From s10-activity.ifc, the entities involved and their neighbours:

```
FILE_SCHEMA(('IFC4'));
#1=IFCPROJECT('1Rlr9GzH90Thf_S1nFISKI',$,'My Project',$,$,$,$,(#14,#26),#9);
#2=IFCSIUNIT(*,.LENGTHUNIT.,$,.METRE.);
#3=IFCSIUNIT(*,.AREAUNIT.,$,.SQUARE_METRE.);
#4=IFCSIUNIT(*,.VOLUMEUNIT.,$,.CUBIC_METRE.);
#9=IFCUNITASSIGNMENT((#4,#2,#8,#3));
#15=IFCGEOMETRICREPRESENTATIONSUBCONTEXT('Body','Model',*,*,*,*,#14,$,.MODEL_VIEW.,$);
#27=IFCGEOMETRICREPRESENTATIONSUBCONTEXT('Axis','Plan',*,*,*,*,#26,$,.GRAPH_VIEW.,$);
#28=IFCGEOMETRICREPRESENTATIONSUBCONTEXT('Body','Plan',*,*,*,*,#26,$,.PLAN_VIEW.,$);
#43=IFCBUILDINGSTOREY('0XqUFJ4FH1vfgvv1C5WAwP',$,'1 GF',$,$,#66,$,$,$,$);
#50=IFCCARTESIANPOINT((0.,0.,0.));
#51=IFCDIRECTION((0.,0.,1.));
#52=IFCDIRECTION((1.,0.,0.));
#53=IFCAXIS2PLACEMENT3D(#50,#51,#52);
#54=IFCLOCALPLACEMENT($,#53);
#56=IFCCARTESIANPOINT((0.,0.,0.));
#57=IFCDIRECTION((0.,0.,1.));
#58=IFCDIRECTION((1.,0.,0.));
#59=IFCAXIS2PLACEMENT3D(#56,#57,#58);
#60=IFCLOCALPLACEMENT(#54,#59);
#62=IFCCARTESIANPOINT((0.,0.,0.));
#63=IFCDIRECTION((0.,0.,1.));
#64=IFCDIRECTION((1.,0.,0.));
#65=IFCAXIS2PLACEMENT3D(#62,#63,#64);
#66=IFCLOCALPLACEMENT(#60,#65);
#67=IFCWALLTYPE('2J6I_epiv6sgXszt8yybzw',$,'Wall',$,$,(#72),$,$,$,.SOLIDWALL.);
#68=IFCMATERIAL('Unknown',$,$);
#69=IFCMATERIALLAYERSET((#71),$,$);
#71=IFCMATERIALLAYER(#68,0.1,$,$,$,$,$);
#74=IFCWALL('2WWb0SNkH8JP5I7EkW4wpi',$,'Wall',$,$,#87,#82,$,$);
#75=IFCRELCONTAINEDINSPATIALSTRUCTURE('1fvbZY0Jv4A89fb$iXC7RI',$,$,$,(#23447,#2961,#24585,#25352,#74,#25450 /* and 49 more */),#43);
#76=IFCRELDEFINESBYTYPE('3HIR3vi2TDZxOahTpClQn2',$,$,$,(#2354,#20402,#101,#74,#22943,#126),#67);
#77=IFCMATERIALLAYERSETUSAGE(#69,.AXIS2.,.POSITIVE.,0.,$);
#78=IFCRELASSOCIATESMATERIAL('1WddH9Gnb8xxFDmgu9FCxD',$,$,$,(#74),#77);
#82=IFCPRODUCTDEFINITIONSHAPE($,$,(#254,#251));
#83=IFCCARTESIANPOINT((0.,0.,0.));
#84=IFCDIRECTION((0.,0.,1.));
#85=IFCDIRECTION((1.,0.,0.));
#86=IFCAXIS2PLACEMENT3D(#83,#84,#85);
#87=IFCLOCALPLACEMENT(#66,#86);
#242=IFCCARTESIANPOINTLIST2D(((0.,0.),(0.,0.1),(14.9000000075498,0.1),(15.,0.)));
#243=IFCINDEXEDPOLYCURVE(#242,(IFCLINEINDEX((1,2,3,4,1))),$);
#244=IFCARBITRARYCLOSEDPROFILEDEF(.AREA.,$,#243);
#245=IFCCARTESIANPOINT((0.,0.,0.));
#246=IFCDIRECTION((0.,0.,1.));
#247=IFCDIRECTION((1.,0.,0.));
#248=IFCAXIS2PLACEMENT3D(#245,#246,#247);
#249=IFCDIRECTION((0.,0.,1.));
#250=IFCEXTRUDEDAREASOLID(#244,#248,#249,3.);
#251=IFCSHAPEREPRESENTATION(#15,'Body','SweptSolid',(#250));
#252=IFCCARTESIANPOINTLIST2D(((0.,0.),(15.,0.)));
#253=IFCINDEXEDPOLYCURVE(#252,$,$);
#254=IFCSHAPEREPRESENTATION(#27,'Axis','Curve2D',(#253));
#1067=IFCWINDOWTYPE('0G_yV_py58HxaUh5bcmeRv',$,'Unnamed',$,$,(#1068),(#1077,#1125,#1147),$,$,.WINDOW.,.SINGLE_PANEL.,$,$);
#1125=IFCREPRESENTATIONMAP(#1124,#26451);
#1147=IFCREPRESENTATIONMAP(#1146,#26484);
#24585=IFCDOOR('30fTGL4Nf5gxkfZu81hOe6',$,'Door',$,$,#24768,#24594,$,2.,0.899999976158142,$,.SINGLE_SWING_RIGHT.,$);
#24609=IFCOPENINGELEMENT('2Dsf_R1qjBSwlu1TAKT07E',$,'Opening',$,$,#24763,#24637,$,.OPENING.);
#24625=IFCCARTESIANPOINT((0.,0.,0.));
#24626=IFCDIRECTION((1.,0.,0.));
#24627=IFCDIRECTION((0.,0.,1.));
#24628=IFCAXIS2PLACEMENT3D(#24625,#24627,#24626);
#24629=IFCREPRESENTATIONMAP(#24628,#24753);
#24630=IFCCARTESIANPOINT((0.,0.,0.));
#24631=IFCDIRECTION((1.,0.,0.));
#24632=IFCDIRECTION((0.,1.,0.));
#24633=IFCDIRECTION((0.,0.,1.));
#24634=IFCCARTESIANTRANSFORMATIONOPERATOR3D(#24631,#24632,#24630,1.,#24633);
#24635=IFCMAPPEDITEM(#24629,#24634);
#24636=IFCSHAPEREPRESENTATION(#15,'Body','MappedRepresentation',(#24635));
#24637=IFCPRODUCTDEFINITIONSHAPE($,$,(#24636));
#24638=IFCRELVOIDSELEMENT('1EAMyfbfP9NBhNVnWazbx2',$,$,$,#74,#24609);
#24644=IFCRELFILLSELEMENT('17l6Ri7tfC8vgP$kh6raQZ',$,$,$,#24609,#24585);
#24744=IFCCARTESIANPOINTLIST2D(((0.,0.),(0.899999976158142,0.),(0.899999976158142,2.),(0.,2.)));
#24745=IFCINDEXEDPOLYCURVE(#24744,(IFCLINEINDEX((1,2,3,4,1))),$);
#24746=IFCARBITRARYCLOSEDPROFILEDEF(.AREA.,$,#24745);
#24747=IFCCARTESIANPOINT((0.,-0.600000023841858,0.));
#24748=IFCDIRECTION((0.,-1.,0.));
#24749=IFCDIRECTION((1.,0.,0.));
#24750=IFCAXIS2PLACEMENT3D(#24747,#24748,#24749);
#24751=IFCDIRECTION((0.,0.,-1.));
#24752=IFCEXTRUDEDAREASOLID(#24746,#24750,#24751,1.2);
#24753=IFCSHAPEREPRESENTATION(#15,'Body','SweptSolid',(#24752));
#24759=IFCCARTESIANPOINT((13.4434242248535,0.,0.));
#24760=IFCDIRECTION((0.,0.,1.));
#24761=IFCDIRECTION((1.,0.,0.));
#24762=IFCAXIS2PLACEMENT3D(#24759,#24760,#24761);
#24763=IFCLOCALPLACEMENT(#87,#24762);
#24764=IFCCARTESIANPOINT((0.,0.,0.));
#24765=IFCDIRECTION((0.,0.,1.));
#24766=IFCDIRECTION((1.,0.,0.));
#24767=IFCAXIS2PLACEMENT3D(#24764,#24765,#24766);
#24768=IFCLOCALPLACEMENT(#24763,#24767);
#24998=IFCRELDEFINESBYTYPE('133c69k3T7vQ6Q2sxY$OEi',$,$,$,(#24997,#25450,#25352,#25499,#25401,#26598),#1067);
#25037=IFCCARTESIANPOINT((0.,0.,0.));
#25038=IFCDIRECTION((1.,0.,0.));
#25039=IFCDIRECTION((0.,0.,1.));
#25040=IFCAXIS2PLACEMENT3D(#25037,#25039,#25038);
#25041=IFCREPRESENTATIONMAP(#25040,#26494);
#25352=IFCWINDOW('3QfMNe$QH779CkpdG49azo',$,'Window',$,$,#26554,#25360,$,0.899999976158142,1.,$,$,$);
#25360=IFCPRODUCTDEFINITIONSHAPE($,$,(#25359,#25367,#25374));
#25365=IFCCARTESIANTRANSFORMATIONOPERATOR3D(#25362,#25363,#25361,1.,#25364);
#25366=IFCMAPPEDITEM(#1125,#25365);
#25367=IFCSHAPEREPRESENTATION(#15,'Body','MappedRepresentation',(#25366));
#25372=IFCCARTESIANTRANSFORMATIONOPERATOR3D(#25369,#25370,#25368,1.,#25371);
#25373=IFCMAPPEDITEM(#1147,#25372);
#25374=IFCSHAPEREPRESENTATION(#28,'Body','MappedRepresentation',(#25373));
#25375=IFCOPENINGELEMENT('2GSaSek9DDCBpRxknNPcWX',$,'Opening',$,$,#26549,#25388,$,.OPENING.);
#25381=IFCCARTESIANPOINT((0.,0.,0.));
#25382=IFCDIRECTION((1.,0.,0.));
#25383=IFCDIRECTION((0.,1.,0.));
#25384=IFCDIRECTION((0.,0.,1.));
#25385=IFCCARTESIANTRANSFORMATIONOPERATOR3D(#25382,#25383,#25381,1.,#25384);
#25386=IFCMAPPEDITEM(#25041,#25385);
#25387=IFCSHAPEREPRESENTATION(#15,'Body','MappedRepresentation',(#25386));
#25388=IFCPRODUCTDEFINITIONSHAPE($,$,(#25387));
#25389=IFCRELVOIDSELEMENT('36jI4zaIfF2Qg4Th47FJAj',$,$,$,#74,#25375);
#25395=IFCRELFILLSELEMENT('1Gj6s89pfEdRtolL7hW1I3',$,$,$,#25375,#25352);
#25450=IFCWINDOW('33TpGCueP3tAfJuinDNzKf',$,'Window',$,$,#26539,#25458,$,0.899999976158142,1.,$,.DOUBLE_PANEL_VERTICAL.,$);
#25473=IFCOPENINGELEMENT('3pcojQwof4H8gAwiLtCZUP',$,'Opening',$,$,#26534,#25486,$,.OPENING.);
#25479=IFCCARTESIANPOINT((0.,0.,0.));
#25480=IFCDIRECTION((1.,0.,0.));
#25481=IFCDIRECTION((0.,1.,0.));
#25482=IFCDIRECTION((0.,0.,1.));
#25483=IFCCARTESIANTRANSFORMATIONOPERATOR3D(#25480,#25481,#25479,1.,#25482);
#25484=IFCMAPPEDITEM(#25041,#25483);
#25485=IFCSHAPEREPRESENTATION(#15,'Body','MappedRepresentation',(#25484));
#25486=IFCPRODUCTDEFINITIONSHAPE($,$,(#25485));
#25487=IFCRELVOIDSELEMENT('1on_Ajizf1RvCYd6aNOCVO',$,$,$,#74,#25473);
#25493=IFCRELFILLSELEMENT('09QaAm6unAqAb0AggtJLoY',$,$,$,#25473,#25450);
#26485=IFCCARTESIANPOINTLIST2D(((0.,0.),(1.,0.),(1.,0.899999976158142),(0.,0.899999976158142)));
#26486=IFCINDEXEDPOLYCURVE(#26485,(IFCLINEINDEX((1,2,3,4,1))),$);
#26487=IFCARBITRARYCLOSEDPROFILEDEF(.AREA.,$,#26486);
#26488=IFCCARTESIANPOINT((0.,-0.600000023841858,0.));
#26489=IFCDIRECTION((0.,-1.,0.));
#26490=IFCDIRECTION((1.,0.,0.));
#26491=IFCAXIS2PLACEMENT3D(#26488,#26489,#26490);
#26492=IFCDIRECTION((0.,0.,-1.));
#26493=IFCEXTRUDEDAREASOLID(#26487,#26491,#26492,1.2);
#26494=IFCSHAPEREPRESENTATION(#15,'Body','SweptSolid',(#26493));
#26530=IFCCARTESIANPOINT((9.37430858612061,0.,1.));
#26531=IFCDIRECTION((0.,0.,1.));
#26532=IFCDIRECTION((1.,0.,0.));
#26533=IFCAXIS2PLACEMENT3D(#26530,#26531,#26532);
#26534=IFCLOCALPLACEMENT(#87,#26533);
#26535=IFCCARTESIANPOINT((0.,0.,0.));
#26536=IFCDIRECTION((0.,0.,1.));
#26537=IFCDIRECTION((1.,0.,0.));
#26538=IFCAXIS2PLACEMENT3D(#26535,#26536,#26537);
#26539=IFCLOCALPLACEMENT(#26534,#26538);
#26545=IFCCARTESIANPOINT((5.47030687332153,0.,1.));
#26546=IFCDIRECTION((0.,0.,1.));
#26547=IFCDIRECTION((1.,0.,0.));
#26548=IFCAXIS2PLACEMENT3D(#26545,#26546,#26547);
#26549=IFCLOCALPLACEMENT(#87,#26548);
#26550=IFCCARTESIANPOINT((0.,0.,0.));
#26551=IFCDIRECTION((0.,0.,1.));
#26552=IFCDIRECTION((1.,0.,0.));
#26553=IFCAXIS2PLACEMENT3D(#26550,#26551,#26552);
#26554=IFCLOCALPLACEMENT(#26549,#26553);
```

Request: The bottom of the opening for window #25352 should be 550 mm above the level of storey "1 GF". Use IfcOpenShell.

```python
import numpy as np
import ifcopenshell
import ifcopenshell.api.geometry
import ifcopenshell.geom
import ifcopenshell.util.element
import ifcopenshell.util.placement
import ifcopenshell.util.shape
import ifcopenshell.util.unit

model = ifcopenshell.open("s10-activity.ifc")
unit_scale = ifcopenshell.util.unit.calculate_unit_scale(model)

window = model.by_guid("3QfMNe$QH779CkpdG49azo")
opening = window.FillsVoids[0].RelatingOpeningElement
storey = ifcopenshell.util.element.get_container(window, ifc_class="IfcBuildingStorey")
level = ifcopenshell.util.placement.get_local_placement(storey.ObjectPlacement)[2, 3]

# The opening's origin need not be at the sill, so measure its lowest point.
shape = ifcopenshell.geom.create_shape(ifcopenshell.geom.settings(), opening)
bottom = ifcopenshell.util.shape.get_shape_bottom_elevation(shape, shape.geometry) / unit_scale
dz = level + 0.55 / unit_scale - bottom

shift = np.array([0.0, 0.0, dz])
# The window is placed relative to its opening, so it follows when the opening moves.
matrix = ifcopenshell.util.placement.get_local_placement(opening.ObjectPlacement)
matrix[:3, 3] += shift
ifcopenshell.api.geometry.edit_object_placement(
    model, product=opening, matrix=matrix, is_si=False, should_transform_children=True
)

print(f"moved by {dz * unit_scale:+.3f} m")

model.write("s10-activity_rev.ifc")
```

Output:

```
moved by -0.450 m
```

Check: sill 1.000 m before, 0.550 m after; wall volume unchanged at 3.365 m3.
